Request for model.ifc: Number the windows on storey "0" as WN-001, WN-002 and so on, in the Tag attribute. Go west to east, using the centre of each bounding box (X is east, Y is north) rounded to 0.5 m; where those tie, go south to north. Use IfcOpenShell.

First a look at what the model holds.

```python
import ifcopenshell
import ifcopenshell.util.element
import ifcopenshell.util.placement

model = ifcopenshell.open("model.ifc")
print(model.schema)
storey = next(s for s in model.by_type("IfcBuildingStorey") if s.Name == "0")
windows = [e for e in ifcopenshell.util.element.get_decomposition(storey) if e.is_a("IfcWindow")]
for e in sorted(windows, key=lambda e: e.id()):
    origin = ifcopenshell.util.placement.get_local_placement(e.ObjectPlacement)[:3, 3]
    print(e.id(), e.Tag, e.Name, origin.round(2) + 0.0, sep=" | ")
```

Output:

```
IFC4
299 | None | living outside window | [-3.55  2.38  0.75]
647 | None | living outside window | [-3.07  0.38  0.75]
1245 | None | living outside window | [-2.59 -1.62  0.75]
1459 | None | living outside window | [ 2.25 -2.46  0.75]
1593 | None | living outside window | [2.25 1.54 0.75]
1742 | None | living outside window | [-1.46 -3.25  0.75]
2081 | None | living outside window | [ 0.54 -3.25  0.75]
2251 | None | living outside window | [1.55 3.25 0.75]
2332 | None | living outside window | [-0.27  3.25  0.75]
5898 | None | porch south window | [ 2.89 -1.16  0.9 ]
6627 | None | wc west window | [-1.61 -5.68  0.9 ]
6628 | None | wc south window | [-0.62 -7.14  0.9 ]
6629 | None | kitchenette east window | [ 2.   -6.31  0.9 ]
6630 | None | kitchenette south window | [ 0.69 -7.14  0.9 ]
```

```python
import ifcopenshell
import ifcopenshell.geom
import ifcopenshell.util.element
import ifcopenshell.util.shape

model = ifcopenshell.open("model.ifc")
settings = ifcopenshell.geom.settings()
settings.set("use-world-coords", True)


def centre(element):
    shape = ifcopenshell.geom.create_shape(settings, element)
    return ifcopenshell.util.shape.get_bbox_centroid(shape.geometry)


storey = next(s for s in model.by_type("IfcBuildingStorey") if s.Name == "0")
windows = [e for e in ifcopenshell.util.element.get_decomposition(storey) if e.is_a("IfcWindow")]

# Insertion points can sit at a corner or the storey origin, so sort by the geometry (in metres).
centres = {e: centre(e) for e in windows}
windows.sort(key=lambda e: (round(centres[e][0] / 0.5), centres[e][1]))

for i, e in enumerate(windows, start=1):
    number = f"WN-0{i:02d}"
    e.Tag = number
    print(e.id(), number)

model.write("model_edited.ifc")
```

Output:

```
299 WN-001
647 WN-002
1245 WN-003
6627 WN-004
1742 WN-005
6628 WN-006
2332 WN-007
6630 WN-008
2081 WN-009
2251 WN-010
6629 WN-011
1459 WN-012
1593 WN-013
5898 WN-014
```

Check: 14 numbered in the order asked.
